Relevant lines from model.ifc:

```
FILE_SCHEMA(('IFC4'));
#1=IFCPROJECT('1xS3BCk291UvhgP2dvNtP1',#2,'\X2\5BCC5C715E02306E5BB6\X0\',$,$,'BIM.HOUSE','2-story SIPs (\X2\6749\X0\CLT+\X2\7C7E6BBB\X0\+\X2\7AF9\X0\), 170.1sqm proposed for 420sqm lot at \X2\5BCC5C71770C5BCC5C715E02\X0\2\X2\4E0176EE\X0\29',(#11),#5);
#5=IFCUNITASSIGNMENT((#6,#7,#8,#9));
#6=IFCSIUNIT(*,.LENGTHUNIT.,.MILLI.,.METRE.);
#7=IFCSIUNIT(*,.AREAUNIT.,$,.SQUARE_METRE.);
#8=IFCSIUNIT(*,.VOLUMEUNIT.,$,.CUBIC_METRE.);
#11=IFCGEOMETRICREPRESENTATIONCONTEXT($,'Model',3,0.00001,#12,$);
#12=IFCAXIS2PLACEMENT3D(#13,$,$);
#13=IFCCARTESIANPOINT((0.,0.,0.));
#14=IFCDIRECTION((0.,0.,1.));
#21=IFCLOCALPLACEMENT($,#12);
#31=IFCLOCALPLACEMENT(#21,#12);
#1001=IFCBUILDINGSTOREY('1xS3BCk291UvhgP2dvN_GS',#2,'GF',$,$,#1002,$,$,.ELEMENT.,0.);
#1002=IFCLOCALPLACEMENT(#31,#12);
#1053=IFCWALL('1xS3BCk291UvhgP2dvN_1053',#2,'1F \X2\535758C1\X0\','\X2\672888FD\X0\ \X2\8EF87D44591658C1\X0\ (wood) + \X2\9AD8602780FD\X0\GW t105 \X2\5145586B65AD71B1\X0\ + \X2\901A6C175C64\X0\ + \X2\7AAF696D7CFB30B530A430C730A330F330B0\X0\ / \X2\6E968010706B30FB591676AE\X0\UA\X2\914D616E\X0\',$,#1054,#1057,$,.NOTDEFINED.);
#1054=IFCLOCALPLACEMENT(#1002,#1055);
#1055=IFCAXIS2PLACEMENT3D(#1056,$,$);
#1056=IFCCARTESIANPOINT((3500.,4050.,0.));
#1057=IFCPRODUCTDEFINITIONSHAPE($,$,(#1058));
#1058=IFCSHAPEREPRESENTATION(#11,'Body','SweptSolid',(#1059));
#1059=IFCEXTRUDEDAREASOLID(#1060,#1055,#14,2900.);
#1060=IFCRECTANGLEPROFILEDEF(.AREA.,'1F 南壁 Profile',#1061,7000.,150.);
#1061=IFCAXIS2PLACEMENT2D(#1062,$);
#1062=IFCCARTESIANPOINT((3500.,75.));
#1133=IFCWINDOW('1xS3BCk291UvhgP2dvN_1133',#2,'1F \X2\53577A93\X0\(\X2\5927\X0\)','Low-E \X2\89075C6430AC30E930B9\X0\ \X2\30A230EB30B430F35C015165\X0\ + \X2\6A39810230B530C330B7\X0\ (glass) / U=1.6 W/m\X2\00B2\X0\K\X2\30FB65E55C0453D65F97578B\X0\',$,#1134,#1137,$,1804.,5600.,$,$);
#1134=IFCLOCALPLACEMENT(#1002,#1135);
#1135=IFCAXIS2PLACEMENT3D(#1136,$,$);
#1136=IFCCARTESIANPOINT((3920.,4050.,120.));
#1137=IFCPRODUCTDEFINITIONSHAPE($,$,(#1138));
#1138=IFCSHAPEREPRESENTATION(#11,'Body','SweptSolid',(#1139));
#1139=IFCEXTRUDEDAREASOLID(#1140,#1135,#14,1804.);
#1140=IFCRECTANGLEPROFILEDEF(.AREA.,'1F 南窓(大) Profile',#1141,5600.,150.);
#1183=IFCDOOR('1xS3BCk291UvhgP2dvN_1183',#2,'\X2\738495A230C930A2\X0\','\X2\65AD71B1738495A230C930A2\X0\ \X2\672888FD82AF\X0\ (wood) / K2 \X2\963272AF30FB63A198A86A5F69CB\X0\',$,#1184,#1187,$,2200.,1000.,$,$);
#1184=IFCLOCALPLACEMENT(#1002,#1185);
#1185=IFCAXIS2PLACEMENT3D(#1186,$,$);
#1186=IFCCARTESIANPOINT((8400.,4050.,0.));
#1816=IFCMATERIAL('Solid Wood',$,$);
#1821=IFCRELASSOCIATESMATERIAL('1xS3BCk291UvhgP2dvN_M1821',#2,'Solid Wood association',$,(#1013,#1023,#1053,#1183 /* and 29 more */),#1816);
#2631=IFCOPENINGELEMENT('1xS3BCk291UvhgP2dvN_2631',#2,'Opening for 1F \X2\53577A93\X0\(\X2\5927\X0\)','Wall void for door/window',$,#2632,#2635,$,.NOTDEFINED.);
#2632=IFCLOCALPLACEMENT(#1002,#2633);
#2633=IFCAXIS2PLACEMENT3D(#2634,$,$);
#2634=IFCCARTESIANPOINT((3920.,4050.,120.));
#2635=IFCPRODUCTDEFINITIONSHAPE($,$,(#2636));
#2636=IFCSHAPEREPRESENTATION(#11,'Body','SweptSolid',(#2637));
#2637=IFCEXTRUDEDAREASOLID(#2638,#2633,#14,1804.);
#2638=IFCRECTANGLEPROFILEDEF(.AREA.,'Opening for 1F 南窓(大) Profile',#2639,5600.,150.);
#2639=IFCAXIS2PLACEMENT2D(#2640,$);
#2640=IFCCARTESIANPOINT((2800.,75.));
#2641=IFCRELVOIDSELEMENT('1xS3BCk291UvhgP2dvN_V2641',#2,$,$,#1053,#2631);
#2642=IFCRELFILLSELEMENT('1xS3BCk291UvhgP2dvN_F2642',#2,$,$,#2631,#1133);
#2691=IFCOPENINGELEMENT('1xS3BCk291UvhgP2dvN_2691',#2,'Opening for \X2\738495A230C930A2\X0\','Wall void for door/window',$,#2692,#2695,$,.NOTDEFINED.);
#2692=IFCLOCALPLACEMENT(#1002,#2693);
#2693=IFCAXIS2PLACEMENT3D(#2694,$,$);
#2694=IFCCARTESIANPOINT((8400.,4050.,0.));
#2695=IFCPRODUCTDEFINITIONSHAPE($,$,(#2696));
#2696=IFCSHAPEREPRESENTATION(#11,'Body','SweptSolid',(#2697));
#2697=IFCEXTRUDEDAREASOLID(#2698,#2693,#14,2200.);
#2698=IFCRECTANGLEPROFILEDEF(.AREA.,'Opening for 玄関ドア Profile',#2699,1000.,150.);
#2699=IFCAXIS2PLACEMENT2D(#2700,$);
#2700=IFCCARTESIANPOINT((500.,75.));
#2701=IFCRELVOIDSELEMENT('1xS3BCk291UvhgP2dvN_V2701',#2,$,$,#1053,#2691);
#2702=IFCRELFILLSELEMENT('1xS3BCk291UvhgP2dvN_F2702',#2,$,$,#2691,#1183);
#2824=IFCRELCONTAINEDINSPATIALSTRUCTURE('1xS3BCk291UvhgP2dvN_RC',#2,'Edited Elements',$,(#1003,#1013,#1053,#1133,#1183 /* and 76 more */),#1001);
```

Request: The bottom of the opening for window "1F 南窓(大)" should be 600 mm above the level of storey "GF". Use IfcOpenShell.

```python
import numpy as np
import ifcopenshell
import ifcopenshell.api.geometry
import ifcopenshell.geom
import ifcopenshell.util.element
import ifcopenshell.util.placement
import ifcopenshell.util.shape
import ifcopenshell.util.unit

model = ifcopenshell.open("model.ifc")
unit_scale = ifcopenshell.util.unit.calculate_unit_scale(model)

window = model.by_guid("1xS3BCk291UvhgP2dvN_1133")
opening = window.FillsVoids[0].RelatingOpeningElement
storey = ifcopenshell.util.element.get_container(window, ifc_class="IfcBuildingStorey")
level = ifcopenshell.util.placement.get_local_placement(storey.ObjectPlacement)[2, 3]

# The opening's origin need not be at the sill, so measure its lowest point.
shape = ifcopenshell.geom.create_shape(ifcopenshell.geom.settings(), opening)
bottom = ifcopenshell.util.shape.get_shape_bottom_elevation(shape, shape.geometry) / unit_scale
dz = level + 600.0 - bottom

shift = np.array([0.0, 0.0, dz])
# The window is not placed relative to its opening, so move both.
for product in (opening, window):
    matrix = ifcopenshell.util.placement.get_local_placement(product.ObjectPlacement)
    matrix[:3, 3] += shift
    ifcopenshell.api.geometry.edit_object_placement(model, product=product, matrix=matrix, is_si=False)

print(f"moved by {dz * unit_scale:+.3f} m")

model.write("model-out.ifc")
```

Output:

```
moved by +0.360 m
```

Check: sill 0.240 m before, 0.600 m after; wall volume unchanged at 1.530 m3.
